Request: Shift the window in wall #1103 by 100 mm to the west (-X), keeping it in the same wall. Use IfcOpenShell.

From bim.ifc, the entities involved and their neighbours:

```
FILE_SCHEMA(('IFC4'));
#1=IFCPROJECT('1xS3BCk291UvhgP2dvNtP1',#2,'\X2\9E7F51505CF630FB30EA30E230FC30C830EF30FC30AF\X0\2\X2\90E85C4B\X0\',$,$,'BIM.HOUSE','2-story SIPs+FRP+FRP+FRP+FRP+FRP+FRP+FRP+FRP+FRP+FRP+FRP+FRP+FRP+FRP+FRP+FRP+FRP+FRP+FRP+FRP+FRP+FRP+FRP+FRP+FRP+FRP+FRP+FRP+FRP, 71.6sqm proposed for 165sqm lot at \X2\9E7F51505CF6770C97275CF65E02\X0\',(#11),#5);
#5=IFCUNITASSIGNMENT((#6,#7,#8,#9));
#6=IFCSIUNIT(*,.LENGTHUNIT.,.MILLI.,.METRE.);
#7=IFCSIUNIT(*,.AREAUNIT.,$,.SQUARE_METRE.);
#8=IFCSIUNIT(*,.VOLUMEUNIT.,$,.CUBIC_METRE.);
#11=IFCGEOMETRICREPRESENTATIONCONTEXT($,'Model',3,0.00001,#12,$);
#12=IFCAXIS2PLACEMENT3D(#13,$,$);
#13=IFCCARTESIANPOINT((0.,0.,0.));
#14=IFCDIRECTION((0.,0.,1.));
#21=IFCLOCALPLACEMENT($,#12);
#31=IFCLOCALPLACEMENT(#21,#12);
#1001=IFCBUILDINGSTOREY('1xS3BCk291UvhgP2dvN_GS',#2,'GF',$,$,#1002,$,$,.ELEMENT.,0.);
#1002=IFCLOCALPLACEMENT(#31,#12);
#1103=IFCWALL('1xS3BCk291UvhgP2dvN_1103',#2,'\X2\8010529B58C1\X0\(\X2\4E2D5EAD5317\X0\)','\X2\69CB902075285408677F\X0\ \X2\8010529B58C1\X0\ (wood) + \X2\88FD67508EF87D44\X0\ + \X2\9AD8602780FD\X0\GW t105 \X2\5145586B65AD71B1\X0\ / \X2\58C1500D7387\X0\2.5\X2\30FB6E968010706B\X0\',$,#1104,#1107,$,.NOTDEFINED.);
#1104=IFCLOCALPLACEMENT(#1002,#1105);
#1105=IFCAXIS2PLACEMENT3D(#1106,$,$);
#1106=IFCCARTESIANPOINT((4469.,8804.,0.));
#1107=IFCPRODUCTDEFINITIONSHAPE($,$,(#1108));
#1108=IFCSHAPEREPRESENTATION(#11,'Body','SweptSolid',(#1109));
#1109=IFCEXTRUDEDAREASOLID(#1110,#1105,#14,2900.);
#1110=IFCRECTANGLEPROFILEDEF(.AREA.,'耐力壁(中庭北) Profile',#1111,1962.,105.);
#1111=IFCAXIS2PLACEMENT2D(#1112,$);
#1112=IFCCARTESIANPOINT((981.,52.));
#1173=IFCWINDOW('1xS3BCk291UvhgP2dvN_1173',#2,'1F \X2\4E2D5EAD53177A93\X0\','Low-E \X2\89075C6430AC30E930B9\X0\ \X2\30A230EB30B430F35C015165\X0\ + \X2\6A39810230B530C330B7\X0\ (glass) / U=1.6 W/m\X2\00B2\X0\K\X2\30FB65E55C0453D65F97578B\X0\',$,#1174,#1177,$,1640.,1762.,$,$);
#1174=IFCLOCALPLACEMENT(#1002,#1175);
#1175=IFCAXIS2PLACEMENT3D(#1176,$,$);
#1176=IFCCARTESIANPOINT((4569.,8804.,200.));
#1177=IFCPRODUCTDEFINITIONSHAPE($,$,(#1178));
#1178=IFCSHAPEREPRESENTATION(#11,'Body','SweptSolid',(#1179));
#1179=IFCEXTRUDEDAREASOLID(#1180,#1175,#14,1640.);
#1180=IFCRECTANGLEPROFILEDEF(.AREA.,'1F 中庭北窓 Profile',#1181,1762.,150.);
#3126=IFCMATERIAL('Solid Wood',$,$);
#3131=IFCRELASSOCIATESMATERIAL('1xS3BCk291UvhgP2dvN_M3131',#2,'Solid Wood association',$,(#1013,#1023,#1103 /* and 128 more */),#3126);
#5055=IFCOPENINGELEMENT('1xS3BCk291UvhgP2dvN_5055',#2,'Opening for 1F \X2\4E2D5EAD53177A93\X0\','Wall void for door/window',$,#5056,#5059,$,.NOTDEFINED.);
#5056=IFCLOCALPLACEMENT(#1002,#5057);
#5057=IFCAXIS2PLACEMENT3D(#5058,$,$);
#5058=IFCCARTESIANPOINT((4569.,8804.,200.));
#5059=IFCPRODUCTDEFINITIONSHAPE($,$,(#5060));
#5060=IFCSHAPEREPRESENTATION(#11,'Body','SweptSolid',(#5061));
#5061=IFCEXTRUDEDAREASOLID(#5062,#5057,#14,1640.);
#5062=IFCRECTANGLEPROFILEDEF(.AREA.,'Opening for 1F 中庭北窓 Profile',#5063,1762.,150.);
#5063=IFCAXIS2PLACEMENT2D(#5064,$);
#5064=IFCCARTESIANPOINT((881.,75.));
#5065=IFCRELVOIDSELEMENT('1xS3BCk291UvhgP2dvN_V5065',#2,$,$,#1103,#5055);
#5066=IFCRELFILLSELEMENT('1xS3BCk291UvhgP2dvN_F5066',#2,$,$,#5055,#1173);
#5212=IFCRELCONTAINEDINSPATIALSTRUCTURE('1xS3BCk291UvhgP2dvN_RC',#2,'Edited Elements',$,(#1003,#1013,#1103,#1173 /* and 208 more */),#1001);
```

```python
import ifcopenshell
import ifcopenshell.api.geometry
import ifcopenshell.util.placement
import ifcopenshell.util.unit

model = ifcopenshell.open("bim.ifc")
unit_scale = ifcopenshell.util.unit.calculate_unit_scale(model)

window = model.by_guid("1xS3BCk291UvhgP2dvN_1173")
opening = window.FillsVoids[0].RelatingOpeningElement
wall = opening.VoidsElements[0].RelatingBuildingElement

wall_matrix = ifcopenshell.util.placement.get_local_placement(wall.ObjectPlacement)
shift = wall_matrix[:3, 0] * -0.1 / unit_scale
before = ifcopenshell.util.placement.get_local_placement(window.ObjectPlacement)[:3, 3].copy()

# The window is not placed relative to its opening, so move both.
for product in (opening, window):
    matrix = ifcopenshell.util.placement.get_local_placement(product.ObjectPlacement)
    matrix[:3, 3] += shift
    ifcopenshell.api.geometry.edit_object_placement(model, product=product, matrix=matrix, is_si=False)

after = ifcopenshell.util.placement.get_local_placement(window.ObjectPlacement)[:3, 3]
print("window moved by", (after - before).round(3) + 0.0)

model.write("bim_v2.ifc")
```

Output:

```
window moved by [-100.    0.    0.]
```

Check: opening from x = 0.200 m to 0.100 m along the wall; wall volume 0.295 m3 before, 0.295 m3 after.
